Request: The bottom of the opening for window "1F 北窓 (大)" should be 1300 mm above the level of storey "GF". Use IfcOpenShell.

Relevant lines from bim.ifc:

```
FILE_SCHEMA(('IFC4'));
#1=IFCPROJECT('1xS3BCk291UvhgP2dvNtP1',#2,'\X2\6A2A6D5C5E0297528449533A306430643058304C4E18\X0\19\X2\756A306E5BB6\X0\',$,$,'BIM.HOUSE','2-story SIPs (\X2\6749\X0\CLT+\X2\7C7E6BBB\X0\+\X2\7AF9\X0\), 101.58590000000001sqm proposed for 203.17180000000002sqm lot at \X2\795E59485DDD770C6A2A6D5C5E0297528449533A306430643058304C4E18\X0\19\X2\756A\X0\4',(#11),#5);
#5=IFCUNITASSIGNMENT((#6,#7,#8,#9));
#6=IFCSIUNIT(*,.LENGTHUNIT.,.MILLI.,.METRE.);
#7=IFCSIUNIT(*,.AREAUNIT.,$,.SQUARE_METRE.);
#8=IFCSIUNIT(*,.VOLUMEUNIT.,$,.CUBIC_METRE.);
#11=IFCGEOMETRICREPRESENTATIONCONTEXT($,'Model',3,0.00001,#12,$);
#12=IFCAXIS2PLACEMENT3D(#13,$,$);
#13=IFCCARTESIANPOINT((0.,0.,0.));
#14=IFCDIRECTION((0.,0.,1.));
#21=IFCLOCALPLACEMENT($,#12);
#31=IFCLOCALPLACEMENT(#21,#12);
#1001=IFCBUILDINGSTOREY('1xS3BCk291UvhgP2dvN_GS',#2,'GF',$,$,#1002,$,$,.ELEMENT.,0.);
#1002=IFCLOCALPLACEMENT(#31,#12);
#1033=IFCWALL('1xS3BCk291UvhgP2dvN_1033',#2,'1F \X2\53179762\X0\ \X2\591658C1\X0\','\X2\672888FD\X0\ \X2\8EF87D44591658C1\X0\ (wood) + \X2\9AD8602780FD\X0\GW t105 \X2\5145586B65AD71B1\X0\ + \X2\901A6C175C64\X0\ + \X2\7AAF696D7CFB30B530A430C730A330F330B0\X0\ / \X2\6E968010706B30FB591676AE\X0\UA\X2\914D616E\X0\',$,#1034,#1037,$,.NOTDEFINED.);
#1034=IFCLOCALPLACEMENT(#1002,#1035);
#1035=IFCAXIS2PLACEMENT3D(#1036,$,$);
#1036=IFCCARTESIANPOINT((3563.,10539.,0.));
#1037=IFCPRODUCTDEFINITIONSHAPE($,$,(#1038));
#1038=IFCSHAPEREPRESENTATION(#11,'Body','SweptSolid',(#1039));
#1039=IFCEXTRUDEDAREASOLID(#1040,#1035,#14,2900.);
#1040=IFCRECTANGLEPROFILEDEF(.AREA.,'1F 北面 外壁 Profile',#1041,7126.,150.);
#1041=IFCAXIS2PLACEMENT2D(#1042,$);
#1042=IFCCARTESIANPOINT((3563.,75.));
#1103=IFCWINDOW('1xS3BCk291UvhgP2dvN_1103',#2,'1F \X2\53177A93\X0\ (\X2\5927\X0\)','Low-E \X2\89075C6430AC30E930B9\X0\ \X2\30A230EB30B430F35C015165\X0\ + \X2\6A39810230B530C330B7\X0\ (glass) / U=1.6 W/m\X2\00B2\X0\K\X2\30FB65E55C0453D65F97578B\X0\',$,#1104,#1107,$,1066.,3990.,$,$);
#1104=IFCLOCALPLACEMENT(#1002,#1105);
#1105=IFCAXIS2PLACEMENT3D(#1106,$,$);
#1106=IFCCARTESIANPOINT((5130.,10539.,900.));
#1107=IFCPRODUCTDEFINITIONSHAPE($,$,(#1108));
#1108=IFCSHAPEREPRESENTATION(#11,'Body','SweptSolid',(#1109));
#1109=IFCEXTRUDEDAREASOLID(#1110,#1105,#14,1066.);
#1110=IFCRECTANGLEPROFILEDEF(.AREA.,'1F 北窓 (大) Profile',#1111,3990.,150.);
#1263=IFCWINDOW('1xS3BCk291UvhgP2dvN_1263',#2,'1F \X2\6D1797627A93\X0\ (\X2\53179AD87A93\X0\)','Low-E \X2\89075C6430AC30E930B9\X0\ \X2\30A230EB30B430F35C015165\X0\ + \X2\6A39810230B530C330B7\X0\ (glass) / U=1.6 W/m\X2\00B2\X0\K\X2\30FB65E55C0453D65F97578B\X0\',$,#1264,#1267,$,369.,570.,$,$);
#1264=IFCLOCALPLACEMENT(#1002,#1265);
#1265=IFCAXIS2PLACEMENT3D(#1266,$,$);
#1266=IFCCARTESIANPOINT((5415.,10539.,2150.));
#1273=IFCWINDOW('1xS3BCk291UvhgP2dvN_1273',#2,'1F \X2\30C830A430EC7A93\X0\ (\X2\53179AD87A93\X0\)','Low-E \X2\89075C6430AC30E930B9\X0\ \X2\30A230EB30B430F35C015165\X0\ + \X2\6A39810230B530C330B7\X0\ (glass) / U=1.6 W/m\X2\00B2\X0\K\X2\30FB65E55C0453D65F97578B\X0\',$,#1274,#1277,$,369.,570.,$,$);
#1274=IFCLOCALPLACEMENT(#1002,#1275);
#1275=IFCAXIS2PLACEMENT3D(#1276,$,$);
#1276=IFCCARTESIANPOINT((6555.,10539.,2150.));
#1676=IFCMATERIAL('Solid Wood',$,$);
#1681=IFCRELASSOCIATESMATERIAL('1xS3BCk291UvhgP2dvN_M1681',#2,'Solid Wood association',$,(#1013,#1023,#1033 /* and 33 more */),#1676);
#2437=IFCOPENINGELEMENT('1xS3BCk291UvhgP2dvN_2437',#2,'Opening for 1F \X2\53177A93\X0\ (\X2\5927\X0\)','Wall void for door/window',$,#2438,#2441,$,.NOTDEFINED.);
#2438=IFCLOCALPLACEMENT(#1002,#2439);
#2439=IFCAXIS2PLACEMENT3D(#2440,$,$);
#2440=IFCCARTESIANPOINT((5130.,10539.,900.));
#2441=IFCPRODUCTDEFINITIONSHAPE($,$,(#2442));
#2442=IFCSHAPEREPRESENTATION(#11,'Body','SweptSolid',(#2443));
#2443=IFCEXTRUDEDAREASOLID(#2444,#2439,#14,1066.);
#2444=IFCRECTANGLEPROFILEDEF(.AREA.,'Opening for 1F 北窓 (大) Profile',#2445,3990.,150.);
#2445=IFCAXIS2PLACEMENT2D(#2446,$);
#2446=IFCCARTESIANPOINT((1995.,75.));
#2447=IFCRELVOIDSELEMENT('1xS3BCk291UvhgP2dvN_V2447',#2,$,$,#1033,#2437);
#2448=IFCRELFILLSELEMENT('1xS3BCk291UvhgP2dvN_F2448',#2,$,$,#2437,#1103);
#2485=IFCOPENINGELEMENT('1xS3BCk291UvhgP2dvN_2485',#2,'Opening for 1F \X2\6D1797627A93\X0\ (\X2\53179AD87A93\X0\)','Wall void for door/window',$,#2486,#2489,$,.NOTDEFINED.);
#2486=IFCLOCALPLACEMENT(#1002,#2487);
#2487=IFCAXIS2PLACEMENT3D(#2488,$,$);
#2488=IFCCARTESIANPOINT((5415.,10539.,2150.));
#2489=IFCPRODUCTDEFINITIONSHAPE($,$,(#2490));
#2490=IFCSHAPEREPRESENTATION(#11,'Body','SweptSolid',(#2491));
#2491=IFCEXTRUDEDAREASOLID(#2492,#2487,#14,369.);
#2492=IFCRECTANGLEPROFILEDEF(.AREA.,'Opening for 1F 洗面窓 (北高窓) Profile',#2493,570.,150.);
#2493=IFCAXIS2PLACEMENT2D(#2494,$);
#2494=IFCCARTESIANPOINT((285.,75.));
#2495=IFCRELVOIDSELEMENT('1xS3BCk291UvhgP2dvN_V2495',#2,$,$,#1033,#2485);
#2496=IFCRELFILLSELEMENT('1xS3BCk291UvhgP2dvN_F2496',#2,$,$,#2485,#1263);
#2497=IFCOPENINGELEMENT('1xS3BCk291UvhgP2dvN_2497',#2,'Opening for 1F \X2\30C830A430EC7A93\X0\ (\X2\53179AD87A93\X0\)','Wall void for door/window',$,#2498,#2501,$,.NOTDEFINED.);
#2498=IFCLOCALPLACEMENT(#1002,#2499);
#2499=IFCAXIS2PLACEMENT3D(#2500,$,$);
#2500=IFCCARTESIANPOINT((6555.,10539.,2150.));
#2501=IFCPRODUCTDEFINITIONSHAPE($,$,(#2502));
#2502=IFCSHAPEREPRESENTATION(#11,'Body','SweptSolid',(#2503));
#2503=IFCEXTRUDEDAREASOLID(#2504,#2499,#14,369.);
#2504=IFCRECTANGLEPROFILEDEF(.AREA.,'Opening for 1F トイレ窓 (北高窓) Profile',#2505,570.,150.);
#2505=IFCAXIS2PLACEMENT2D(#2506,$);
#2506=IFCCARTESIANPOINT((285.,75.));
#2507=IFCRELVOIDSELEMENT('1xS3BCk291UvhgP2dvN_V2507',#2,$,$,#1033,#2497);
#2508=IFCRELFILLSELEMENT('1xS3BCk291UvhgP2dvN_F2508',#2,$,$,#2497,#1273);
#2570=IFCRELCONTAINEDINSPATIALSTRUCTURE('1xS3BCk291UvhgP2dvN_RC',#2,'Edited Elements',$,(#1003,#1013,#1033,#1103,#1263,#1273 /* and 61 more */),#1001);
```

```python
import numpy as np
import ifcopenshell
import ifcopenshell.api.geometry
import ifcopenshell.geom
import ifcopenshell.util.element
import ifcopenshell.util.placement
import ifcopenshell.util.shape
import ifcopenshell.util.unit

model = ifcopenshell.open("bim.ifc")
unit_scale = ifcopenshell.util.unit.calculate_unit_scale(model)

window = model.by_guid("1xS3BCk291UvhgP2dvN_1103")
opening = window.FillsVoids[0].RelatingOpeningElement
storey = ifcopenshell.util.element.get_container(window, ifc_class="IfcBuildingStorey")
level = ifcopenshell.util.placement.get_local_placement(storey.ObjectPlacement)[2, 3]

# The opening's origin need not be at the sill, so measure its lowest point.
shape = ifcopenshell.geom.create_shape(ifcopenshell.geom.settings(), opening)
bottom = ifcopenshell.util.shape.get_shape_bottom_elevation(shape, shape.geometry) / unit_scale
dz = level + 1.3 / unit_scale - bottom

shift = np.array([0.0, 0.0, dz])
# The window is not placed relative to its opening, so move both.
for product in (opening, window):
    matrix = ifcopenshell.util.placement.get_local_placement(product.ObjectPlacement)
    matrix[:3, 3] += shift
    ifcopenshell.api.geometry.edit_object_placement(model, product=product, matrix=matrix, is_si=False)

print(f"moved by {dz * unit_scale:+.3f} m")

model.write("bim_edited.ifc")
```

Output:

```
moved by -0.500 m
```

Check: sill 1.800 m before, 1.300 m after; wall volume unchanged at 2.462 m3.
